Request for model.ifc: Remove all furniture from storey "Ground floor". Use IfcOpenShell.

First a look at what the model holds.

```python
import ifcopenshell
import ifcopenshell.util.element

model = ifcopenshell.open("model.ifc")
print(model.schema)
storey = next(s for s in model.by_type("IfcBuildingStorey") if s.Name == "Ground floor")
furniture = [e for e in ifcopenshell.util.element.get_decomposition(storey) if e.is_a("IfcFurnishingElement")]
seen = {}
for e in furniture:
    element_type = ifcopenshell.util.element.get_type(e)
    name = element_type.Name if element_type not in (None, e) else None
    seen[name] = seen.get(name, 0) + 1
for name, count in sorted(seen.items(), key=str):
    print(count, "x", name)
```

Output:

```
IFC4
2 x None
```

```python
import ifcopenshell
import ifcopenshell.api.root
import ifcopenshell.util.element

model = ifcopenshell.open("model.ifc")

storey = next(s for s in model.by_type("IfcBuildingStorey") if s.Name == "Ground floor")
furniture = [e for e in ifcopenshell.util.element.get_decomposition(storey) if e.is_a("IfcFurnishingElement")]

for e in furniture:
    ifcopenshell.api.root.remove_product(model, product=e)
print(len(furniture), "removed")

model.write("model_v2.ifc")
```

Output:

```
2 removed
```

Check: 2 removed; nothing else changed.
